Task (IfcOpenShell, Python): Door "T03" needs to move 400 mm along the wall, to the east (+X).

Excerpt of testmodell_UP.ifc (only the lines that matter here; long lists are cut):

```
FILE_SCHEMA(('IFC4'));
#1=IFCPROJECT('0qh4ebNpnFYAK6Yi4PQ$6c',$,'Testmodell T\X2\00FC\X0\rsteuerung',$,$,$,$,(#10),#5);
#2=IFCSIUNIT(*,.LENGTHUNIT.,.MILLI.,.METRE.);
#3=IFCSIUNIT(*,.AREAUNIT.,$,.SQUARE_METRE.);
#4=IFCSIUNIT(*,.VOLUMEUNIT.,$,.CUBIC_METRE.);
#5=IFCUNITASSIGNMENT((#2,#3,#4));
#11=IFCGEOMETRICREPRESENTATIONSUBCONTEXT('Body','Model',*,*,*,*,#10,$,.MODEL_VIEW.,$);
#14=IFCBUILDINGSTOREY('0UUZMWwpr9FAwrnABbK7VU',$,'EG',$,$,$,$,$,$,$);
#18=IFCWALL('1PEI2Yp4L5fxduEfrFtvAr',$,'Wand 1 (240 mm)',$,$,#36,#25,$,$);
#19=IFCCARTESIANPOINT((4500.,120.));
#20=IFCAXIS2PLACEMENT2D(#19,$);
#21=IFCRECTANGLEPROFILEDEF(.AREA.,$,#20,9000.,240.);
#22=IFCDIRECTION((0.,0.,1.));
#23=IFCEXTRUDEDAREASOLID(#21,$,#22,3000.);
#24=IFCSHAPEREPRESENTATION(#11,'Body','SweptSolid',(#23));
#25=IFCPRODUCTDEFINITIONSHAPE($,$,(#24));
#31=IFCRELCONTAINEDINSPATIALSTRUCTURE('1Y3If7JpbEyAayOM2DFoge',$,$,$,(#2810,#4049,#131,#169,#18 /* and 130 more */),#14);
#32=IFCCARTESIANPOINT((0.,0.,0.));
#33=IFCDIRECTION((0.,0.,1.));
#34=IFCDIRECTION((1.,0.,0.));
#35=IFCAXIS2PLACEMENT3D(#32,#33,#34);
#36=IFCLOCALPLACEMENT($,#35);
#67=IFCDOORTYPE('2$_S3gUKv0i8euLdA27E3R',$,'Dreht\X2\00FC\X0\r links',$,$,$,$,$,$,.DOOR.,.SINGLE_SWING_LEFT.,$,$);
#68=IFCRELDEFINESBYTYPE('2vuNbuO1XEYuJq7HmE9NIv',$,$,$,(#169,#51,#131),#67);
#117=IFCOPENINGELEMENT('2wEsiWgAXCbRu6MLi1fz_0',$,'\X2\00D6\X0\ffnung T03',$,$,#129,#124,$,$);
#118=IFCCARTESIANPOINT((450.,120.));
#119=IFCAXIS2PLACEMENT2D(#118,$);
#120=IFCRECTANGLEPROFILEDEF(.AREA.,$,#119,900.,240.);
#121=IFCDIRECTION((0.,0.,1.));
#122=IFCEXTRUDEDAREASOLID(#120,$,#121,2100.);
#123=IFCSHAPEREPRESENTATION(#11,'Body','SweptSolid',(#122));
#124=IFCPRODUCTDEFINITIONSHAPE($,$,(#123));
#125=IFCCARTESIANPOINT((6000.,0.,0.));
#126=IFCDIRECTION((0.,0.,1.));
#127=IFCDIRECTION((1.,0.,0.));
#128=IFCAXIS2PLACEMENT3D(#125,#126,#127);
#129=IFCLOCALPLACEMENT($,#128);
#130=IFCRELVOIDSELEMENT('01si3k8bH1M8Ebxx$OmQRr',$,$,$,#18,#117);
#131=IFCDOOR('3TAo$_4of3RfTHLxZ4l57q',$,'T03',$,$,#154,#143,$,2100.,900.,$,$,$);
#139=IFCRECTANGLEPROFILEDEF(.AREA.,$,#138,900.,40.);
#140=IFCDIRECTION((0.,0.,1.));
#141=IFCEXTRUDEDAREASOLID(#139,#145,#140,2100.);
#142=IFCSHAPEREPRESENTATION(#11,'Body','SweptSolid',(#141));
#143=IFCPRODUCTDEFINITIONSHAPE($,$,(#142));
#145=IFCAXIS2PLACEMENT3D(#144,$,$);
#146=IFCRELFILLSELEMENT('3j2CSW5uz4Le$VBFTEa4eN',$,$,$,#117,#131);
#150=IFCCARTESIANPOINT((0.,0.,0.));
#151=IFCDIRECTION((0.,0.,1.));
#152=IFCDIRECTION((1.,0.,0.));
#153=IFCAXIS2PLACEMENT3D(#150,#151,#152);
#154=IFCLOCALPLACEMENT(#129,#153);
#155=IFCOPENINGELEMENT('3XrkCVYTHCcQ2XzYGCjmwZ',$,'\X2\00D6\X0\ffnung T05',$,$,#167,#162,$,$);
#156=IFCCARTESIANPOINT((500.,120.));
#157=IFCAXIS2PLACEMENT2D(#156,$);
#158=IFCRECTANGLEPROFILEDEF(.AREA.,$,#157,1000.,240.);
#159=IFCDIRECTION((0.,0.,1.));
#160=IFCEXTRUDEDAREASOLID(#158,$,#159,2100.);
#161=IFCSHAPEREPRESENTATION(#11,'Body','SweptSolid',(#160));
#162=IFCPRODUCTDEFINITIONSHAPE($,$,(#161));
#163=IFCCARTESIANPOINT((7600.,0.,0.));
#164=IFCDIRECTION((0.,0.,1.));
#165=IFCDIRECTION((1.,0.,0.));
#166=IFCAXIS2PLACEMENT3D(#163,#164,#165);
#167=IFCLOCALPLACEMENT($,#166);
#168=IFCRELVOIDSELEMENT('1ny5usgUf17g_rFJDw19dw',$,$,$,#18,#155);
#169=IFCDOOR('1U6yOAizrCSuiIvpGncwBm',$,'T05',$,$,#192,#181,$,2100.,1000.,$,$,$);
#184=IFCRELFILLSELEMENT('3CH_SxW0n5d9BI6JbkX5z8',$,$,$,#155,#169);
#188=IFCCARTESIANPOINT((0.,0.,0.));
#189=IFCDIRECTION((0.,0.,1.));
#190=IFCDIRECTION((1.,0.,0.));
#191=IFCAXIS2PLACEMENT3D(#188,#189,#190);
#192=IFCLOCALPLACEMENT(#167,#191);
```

```python
import ifcopenshell
import ifcopenshell.api.geometry
import ifcopenshell.util.placement
import ifcopenshell.util.unit

model = ifcopenshell.open("testmodell_UP.ifc")
unit_scale = ifcopenshell.util.unit.calculate_unit_scale(model)

door = model.by_guid("3TAo$_4of3RfTHLxZ4l57q")
opening = door.FillsVoids[0].RelatingOpeningElement
wall = opening.VoidsElements[0].RelatingBuildingElement

wall_matrix = ifcopenshell.util.placement.get_local_placement(wall.ObjectPlacement)
shift = wall_matrix[:3, 0] * 0.4 / unit_scale
before = ifcopenshell.util.placement.get_local_placement(door.ObjectPlacement)[:3, 3].copy()

# The door is placed relative to its opening, so it follows when the opening moves.
matrix = ifcopenshell.util.placement.get_local_placement(opening.ObjectPlacement)
matrix[:3, 3] += shift
ifcopenshell.api.geometry.edit_object_placement(
    model, product=opening, matrix=matrix, is_si=False, should_transform_children=True
)

after = ifcopenshell.util.placement.get_local_placement(door.ObjectPlacement)[:3, 3]
print("door moved by", (after - before).round(3) + 0.0)

model.write("testmodell_UP-out.ifc")
```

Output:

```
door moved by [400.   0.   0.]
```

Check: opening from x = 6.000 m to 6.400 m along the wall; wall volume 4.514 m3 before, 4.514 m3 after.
